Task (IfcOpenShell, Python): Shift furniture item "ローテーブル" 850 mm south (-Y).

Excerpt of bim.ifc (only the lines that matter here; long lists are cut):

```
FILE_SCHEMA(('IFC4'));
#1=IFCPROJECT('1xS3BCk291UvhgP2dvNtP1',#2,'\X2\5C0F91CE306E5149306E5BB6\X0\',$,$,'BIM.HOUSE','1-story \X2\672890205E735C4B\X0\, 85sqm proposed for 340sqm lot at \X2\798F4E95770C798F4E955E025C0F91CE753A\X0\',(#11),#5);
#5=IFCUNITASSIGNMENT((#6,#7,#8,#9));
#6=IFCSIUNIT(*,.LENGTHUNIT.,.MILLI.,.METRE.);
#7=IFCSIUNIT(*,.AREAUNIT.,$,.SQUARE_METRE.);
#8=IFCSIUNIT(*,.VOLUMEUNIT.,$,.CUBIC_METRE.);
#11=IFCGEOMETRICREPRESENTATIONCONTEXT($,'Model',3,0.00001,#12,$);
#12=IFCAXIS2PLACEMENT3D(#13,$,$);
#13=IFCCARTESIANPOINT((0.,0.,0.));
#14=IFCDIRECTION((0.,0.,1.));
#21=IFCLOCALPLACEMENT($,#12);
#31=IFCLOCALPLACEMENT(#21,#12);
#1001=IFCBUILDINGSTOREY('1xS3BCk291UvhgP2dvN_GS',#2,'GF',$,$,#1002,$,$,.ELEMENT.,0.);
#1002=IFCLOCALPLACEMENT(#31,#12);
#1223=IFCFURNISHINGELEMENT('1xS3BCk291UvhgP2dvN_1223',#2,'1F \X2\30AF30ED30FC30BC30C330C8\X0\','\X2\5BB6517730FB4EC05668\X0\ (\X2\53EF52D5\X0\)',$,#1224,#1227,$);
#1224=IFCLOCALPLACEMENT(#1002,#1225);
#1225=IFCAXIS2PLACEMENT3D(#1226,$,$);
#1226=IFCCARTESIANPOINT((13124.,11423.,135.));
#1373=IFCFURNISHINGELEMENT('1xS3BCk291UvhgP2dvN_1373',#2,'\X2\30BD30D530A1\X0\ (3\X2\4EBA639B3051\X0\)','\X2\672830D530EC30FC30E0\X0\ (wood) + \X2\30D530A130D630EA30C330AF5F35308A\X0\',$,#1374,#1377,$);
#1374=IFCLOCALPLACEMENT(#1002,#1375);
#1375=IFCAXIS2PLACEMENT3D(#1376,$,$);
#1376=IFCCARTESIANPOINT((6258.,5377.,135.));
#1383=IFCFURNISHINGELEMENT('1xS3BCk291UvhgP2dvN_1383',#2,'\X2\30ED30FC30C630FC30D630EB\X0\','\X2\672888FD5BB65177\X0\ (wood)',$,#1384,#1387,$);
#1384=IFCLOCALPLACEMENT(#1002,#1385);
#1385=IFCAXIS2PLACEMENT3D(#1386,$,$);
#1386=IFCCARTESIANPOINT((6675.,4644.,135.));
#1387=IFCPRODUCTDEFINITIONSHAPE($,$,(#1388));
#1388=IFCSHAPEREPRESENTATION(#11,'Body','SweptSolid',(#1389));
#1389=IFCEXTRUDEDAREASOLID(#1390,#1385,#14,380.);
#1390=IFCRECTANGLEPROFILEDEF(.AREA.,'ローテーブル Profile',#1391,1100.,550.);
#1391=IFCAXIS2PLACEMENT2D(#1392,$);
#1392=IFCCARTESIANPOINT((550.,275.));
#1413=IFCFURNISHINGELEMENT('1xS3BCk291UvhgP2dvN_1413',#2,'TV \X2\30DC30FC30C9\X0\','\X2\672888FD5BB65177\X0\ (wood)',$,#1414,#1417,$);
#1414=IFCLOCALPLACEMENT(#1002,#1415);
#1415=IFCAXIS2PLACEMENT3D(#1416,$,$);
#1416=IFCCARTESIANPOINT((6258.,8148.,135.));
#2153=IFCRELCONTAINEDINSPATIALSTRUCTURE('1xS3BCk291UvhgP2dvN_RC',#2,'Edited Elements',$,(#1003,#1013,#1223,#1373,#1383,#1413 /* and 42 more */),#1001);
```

```python
import ifcopenshell
import ifcopenshell.api.geometry
import ifcopenshell.util.placement
import ifcopenshell.util.unit

model = ifcopenshell.open("bim.ifc")
unit_scale = ifcopenshell.util.unit.calculate_unit_scale(model)

item = model.by_guid("1xS3BCk291UvhgP2dvN_1383")
matrix = ifcopenshell.util.placement.get_local_placement(item.ObjectPlacement)
matrix[1, 3] -= 0.85 / unit_scale
ifcopenshell.api.geometry.edit_object_placement(model, product=item, matrix=matrix, is_si=False)

print(ifcopenshell.util.placement.get_local_placement(item.ObjectPlacement).round(3) + 0.0)

model.write("bim_updated.ifc")
```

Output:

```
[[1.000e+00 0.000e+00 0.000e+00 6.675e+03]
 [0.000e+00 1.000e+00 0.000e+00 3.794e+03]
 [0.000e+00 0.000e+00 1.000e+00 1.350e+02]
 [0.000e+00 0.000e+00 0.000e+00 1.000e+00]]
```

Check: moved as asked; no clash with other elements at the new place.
